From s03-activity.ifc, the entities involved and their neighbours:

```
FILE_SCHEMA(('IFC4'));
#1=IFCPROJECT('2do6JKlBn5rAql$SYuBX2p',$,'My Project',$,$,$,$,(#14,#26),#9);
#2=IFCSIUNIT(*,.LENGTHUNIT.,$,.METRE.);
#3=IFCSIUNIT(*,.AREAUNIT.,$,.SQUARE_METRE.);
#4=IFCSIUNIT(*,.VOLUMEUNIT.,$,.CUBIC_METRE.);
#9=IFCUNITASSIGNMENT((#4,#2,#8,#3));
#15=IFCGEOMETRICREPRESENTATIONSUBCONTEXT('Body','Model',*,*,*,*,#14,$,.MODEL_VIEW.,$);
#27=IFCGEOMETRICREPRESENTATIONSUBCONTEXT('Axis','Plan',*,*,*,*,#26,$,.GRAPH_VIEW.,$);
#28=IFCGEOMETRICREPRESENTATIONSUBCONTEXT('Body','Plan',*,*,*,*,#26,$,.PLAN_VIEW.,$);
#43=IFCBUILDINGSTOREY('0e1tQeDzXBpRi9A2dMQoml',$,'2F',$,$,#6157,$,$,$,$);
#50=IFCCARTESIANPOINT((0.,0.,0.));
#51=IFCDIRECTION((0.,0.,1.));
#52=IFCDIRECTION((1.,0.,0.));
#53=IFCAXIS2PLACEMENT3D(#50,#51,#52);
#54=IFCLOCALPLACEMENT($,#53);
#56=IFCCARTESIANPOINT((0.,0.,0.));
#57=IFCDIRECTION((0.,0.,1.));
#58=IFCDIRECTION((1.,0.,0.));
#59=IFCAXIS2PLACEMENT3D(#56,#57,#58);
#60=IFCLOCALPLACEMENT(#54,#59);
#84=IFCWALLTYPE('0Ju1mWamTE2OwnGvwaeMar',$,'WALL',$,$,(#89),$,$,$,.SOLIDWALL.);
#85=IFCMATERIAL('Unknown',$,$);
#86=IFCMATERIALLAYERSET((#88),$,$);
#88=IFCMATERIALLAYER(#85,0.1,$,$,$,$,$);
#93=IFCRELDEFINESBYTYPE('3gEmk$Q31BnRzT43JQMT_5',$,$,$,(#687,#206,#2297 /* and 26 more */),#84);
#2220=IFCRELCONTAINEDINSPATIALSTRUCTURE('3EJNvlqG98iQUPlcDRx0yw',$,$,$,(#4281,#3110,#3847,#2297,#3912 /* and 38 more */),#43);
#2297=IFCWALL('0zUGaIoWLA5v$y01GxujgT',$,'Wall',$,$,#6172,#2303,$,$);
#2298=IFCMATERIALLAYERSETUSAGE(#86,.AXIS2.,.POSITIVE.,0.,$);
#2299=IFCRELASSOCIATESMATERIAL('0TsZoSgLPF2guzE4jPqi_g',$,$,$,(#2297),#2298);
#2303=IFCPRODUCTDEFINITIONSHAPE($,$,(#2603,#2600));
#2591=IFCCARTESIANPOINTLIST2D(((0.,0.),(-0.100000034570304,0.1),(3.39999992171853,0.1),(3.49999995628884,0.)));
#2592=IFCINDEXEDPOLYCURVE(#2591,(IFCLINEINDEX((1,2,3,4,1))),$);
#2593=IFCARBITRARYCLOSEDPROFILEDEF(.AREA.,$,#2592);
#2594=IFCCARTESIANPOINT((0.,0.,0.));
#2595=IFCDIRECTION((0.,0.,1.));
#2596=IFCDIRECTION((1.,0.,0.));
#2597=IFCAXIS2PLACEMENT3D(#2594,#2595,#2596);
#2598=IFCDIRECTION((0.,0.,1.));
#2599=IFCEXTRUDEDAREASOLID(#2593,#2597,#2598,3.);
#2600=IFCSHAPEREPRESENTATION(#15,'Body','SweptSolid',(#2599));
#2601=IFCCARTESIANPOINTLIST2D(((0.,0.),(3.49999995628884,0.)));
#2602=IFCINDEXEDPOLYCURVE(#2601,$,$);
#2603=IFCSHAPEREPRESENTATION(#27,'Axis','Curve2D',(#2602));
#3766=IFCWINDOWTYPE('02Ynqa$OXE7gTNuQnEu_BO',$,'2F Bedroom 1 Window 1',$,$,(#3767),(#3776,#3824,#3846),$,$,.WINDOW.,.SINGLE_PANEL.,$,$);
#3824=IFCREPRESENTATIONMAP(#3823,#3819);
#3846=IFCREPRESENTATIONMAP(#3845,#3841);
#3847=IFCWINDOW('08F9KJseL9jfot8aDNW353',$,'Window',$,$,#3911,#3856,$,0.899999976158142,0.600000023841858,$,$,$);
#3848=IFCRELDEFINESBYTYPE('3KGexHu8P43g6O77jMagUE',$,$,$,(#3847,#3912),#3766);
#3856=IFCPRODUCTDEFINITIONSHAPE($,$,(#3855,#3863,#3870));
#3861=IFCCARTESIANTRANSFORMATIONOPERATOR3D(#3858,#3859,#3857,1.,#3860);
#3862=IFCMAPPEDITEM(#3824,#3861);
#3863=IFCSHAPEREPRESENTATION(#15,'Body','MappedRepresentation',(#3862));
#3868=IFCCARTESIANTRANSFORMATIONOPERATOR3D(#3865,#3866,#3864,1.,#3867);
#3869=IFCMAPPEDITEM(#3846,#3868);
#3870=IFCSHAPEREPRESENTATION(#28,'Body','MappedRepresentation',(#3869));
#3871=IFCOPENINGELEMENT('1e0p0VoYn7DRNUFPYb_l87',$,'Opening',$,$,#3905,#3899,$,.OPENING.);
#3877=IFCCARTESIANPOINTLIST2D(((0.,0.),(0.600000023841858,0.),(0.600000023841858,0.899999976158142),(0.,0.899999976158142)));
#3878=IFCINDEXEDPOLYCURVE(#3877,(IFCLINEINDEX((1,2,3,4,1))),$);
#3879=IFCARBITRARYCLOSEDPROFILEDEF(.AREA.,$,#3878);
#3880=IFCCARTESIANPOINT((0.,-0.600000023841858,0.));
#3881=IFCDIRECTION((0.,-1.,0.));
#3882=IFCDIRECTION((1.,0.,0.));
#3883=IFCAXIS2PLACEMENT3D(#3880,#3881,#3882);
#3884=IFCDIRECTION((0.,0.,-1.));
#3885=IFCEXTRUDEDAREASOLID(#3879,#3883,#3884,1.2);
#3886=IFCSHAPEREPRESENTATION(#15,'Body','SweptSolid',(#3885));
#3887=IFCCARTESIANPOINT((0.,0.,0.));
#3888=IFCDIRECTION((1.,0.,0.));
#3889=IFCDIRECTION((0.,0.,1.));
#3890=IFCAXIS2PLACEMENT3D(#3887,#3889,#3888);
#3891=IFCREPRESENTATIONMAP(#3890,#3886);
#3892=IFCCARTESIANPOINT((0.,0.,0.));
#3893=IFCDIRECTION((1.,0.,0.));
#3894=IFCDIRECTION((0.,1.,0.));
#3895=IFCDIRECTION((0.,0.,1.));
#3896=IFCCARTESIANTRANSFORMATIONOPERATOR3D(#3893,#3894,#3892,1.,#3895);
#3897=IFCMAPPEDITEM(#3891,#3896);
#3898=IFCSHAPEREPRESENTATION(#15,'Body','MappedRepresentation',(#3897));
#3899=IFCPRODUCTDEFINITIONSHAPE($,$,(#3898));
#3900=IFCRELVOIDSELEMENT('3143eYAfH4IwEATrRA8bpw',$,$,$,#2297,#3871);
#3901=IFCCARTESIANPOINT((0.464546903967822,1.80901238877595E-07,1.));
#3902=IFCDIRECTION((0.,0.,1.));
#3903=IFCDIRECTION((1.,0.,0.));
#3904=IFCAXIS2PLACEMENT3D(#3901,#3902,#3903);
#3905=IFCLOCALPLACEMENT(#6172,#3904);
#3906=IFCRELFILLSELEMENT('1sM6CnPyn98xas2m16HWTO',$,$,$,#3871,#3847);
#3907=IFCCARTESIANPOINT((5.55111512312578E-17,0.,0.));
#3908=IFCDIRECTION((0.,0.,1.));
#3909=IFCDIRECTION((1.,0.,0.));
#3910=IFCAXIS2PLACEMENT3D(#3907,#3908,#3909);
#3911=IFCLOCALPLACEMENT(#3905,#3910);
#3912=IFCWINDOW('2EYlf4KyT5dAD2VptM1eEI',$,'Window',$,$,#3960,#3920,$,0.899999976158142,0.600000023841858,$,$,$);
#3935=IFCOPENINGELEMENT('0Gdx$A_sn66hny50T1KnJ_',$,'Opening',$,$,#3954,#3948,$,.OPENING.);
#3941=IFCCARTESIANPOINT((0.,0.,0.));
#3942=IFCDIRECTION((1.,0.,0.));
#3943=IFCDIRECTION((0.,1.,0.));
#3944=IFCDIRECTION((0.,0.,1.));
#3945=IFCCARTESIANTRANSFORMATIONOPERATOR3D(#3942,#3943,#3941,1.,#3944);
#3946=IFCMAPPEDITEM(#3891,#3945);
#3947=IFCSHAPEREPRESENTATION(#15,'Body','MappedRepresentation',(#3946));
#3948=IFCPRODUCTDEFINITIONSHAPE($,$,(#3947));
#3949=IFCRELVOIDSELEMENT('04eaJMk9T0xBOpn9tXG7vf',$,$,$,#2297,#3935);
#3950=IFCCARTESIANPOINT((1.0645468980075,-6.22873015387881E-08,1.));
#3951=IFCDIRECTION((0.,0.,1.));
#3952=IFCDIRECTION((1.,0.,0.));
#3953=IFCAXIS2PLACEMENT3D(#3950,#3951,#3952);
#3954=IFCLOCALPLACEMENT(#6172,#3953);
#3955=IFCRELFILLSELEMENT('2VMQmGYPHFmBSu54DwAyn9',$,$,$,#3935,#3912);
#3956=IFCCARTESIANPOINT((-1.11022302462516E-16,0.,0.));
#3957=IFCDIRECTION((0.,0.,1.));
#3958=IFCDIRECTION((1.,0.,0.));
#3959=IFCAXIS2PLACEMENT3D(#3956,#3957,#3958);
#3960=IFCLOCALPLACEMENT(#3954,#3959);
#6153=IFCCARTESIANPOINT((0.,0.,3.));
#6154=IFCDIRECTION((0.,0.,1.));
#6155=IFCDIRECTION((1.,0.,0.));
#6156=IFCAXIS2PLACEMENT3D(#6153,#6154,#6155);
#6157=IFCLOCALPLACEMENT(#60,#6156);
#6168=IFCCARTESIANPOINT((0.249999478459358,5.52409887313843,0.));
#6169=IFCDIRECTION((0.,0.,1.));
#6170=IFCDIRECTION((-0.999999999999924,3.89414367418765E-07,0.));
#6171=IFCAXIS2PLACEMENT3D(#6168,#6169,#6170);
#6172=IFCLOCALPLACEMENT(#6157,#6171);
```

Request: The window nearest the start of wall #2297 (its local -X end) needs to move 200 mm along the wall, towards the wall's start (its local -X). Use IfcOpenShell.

```python
import ifcopenshell
import ifcopenshell.api.geometry
import ifcopenshell.util.placement
import ifcopenshell.util.unit

model = ifcopenshell.open("s03-activity.ifc")
unit_scale = ifcopenshell.util.unit.calculate_unit_scale(model)

window = model.by_guid("08F9KJseL9jfot8aDNW353")
opening = window.FillsVoids[0].RelatingOpeningElement
wall = opening.VoidsElements[0].RelatingBuildingElement

wall_matrix = ifcopenshell.util.placement.get_local_placement(wall.ObjectPlacement)
shift = wall_matrix[:3, 0] * -0.2 / unit_scale
before = ifcopenshell.util.placement.get_local_placement(window.ObjectPlacement)[:3, 3].copy()

# The window is placed relative to its opening, so it follows when the opening moves.
matrix = ifcopenshell.util.placement.get_local_placement(opening.ObjectPlacement)
matrix[:3, 3] += shift
ifcopenshell.api.geometry.edit_object_placement(
    model, product=opening, matrix=matrix, is_si=False, should_transform_children=True
)

after = ifcopenshell.util.placement.get_local_placement(window.ObjectPlacement)[:3, 3]
print("window moved by", (after - before).round(3) + 0.0)

model.write("s03-activity_updated.ifc")
```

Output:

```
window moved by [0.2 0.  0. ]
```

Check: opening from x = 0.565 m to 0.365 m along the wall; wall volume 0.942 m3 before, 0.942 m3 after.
